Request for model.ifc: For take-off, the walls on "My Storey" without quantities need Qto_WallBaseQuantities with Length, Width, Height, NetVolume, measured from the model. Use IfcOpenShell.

First a look at what the model holds.

```python
import ifcopenshell
import ifcopenshell.util.element
import ifcopenshell.util.unit

model = ifcopenshell.open("model.ifc")
print(model.schema)
for unit_type in ("LENGTHUNIT", "AREAUNIT", "VOLUMEUNIT"):
    print(unit_type, ifcopenshell.util.unit.calculate_unit_scale(model, unit_type))
storey = next(s for s in model.by_type("IfcBuildingStorey") if s.Name == "My Storey")
walls = [e for e in ifcopenshell.util.element.get_decomposition(storey) if e.is_a("IfcWall")]
for e in sorted(walls, key=lambda e: e.id()):
    print(e.id(), e.is_a(), e.Name, list(ifcopenshell.util.element.get_psets(e, qtos_only=True)), sep=" | ")
```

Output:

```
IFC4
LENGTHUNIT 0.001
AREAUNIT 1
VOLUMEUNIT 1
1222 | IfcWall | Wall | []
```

```python
import ifcopenshell
import ifcopenshell.api.pset
import ifcopenshell.geom
import ifcopenshell.util.element
import ifcopenshell.util.shape
import ifcopenshell.util.unit

model = ifcopenshell.open("model.ifc")
unit_scale = ifcopenshell.util.unit.calculate_unit_scale(model)
volume_scale = ifcopenshell.util.unit.calculate_unit_scale(model, "VOLUMEUNIT")
settings = ifcopenshell.geom.settings()

storey = next(s for s in model.by_type("IfcBuildingStorey") if s.Name == "My Storey")
walls = [e for e in ifcopenshell.util.element.get_decomposition(storey) if e.is_a("IfcWall")]

for e in sorted(walls, key=lambda e: e.id()):
    if ifcopenshell.util.element.get_psets(e, qtos_only=True, should_inherit=False):
        continue
    # Geometry comes back in metres, in the element's own axes.
    shape = ifcopenshell.geom.create_shape(settings, e)
    values = {
        "Length": ifcopenshell.util.shape.get_x(shape.geometry) / unit_scale,
        "Width": ifcopenshell.util.shape.get_y(shape.geometry) / unit_scale,
        "Height": ifcopenshell.util.shape.get_z(shape.geometry) / unit_scale,
        "NetVolume": ifcopenshell.util.shape.get_volume(shape.geometry) / volume_scale,
    }
    qto = ifcopenshell.api.pset.add_qto(model, product=e, name="Qto_WallBaseQuantities")
    ifcopenshell.api.pset.edit_qto(model, qto=qto, properties=values)
    print(e.id(), {k: round(v, 3) for k, v in values.items()})

model.write("model_rev.ifc")
```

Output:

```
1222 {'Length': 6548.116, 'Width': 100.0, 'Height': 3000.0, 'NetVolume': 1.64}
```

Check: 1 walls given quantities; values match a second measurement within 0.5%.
